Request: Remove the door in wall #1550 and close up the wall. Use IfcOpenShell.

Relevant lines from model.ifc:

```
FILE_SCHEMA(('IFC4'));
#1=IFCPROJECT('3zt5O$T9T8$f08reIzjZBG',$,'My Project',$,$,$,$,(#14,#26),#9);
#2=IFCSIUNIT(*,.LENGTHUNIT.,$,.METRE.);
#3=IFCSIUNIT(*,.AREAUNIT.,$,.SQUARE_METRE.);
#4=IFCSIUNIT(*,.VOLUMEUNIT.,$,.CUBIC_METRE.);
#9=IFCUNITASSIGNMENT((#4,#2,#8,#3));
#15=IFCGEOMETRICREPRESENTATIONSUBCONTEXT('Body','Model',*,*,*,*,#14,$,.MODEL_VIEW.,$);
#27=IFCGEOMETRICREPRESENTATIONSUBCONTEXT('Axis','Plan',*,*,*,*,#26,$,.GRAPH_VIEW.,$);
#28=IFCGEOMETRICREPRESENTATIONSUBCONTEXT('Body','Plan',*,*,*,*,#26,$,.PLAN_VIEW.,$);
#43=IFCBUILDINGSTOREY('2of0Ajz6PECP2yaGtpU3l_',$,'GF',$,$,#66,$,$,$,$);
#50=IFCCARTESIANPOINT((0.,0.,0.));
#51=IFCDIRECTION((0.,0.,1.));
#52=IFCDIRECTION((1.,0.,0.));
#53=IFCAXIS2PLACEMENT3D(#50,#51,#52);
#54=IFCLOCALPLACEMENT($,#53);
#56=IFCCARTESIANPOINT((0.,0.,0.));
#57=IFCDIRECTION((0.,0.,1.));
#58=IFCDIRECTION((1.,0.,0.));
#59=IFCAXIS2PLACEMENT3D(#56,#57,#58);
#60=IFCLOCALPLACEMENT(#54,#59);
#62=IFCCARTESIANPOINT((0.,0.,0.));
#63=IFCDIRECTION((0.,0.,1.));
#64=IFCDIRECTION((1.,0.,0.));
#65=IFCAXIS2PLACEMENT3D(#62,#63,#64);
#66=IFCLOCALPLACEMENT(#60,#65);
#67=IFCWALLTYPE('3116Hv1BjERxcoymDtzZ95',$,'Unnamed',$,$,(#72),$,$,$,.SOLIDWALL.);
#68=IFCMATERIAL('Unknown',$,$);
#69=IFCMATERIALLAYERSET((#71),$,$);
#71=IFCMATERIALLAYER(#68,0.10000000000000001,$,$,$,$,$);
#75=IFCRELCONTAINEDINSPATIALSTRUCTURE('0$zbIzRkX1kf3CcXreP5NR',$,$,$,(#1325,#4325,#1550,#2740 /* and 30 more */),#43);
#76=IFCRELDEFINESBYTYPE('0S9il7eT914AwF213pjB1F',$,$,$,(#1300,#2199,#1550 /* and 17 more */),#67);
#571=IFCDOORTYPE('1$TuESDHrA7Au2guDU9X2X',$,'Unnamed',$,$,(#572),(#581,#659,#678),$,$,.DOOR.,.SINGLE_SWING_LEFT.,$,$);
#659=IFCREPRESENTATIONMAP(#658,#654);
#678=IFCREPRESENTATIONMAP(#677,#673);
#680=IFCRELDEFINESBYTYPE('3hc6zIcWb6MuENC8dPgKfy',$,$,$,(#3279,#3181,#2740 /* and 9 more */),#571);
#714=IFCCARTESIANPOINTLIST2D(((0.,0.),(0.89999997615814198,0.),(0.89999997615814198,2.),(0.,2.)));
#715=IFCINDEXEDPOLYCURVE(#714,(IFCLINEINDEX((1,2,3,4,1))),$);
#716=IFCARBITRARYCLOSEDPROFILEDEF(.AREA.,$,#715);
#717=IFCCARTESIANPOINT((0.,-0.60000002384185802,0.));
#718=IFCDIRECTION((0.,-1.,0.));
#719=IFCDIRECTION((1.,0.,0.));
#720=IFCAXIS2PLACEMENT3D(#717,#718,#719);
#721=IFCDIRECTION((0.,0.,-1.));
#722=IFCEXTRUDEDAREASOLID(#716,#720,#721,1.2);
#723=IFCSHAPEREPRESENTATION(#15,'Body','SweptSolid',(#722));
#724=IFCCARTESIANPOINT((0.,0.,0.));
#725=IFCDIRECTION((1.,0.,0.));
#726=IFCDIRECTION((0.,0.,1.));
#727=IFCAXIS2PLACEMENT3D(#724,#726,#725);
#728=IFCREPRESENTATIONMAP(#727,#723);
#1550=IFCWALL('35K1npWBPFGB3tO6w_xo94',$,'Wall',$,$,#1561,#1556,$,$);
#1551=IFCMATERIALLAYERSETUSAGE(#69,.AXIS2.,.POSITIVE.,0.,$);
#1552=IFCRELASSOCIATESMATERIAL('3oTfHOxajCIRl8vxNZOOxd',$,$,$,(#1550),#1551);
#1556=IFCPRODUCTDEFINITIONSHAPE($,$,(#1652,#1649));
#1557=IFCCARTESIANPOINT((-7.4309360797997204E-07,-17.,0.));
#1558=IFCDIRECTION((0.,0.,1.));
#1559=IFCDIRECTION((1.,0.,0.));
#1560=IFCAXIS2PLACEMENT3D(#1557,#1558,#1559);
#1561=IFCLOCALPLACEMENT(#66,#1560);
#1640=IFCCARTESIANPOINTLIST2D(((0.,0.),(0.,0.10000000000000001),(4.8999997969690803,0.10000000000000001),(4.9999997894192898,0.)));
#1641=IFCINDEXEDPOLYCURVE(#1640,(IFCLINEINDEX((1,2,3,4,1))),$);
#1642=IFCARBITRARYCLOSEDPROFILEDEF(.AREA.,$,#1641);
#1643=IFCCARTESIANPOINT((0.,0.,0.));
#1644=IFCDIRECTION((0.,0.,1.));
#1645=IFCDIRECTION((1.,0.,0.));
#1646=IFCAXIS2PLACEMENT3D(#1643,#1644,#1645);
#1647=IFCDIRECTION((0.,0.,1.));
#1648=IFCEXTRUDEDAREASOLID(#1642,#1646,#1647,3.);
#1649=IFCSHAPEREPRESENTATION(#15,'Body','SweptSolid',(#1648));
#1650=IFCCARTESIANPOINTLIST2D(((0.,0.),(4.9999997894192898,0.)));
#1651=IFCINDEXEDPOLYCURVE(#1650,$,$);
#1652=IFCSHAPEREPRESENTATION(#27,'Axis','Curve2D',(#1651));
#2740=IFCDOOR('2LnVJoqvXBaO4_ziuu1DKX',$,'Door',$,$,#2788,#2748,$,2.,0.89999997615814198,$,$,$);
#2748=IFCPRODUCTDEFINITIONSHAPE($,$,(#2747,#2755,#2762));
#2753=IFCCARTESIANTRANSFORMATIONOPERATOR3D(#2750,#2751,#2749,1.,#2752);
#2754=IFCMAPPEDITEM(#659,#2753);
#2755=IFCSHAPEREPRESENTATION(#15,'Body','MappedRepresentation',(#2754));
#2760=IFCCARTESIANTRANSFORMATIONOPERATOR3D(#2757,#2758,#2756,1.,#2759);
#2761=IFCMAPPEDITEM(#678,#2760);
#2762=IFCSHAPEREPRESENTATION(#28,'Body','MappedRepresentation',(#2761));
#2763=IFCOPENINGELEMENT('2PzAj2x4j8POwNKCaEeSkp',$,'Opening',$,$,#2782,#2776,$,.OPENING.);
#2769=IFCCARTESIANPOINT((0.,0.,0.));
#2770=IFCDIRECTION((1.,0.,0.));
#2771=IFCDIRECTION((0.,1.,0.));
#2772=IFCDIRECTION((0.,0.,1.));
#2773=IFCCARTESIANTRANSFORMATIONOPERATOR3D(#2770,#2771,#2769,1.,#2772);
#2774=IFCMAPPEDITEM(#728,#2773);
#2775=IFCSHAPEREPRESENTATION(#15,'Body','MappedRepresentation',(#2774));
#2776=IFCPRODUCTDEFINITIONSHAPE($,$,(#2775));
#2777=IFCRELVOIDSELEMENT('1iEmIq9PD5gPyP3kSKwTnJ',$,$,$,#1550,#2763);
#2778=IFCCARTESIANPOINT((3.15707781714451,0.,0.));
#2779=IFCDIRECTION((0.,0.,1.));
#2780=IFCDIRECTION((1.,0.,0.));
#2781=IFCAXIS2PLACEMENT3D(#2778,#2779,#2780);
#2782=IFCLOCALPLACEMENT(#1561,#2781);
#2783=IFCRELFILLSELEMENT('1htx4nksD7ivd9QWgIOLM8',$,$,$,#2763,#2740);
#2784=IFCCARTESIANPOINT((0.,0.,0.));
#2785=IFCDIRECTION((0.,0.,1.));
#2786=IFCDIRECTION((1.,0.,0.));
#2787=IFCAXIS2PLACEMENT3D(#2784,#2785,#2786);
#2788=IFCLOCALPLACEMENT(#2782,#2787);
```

```python
import ifcopenshell
import ifcopenshell.api.feature
import ifcopenshell.api.root
import ifcopenshell.geom
import ifcopenshell.util.shape

model = ifcopenshell.open("model.ifc")
settings = ifcopenshell.geom.settings()


def volume(element):
    """Net volume in cubic metres, openings subtracted."""
    shape = ifcopenshell.geom.create_shape(settings, element)
    return ifcopenshell.util.shape.get_volume(shape.geometry)


door = model.by_id(2740)
opening = door.FillsVoids[0].RelatingOpeningElement
wall = opening.VoidsElements[0].RelatingBuildingElement
before = volume(wall)

ifcopenshell.api.root.remove_product(model, product=door)
ifcopenshell.api.feature.remove_feature(model, feature=opening)

after = volume(wall)

print(f"wall volume {before:.3f} -> {after:.3f} m3")

model.write("model_updated.ifc")
```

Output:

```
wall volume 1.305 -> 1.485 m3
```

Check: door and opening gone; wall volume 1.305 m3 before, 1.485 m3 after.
